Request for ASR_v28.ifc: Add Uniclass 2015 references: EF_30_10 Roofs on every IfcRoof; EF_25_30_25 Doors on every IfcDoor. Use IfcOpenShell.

First a look at what the model holds.

```python
import ifcopenshell

model = ifcopenshell.open("ASR_v28.ifc")
print(model.schema)
print("classifications:", [c.Name for c in model.by_type("IfcClassification")])
for ifc_class in ("IfcDoor", "IfcRoof", "IfcStair", "IfcWall", "IfcWindow"):
    print(ifc_class, len(model.by_type(ifc_class)))
```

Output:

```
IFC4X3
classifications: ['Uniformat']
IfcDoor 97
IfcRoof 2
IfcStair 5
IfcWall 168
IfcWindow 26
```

```python
import ifcopenshell
import ifcopenshell.api.classification

model = ifcopenshell.open("ASR_v28.ifc")

system = ifcopenshell.api.classification.add_classification(model, classification="Uniclass 2015")

codes = {
    "IfcRoof": ("EF_30_10", "Roofs"),
    "IfcDoor": ("EF_25_30_25", "Doors"),
}
for ifc_class, (code, name) in codes.items():
    products = model.by_type(ifc_class)
    ifcopenshell.api.classification.add_reference(
        model, products=products, classification=system, identification=code, name=name
    )
    print(code, len(products))

model.write("ASR_v28-out.ifc")
```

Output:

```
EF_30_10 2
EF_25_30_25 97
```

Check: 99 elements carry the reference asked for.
